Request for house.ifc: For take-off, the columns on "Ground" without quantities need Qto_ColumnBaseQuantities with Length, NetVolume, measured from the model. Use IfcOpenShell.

First a look at what the model holds.

```python
import ifcopenshell
import ifcopenshell.util.element
import ifcopenshell.util.unit

model = ifcopenshell.open("house.ifc")
print(model.schema)
for unit_type in ("LENGTHUNIT", "AREAUNIT", "VOLUMEUNIT"):
    print(unit_type, ifcopenshell.util.unit.calculate_unit_scale(model, unit_type))
storey = next(s for s in model.by_type("IfcBuildingStorey") if s.Name == "Ground")
columns = [e for e in ifcopenshell.util.element.get_decomposition(storey) if e.is_a("IfcColumn")]
for e in sorted(columns, key=lambda e: e.id()):
    print(e.id(), e.is_a(), e.Name, list(ifcopenshell.util.element.get_psets(e, qtos_only=True)), sep=" | ")
```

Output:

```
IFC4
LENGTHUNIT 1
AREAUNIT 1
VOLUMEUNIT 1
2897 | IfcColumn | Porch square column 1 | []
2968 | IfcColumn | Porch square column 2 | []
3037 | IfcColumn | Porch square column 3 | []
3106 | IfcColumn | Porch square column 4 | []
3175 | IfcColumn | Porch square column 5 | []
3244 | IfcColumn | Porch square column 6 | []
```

```python
import ifcopenshell
import ifcopenshell.api.pset
import ifcopenshell.geom
import ifcopenshell.util.element
import ifcopenshell.util.shape
import ifcopenshell.util.unit

model = ifcopenshell.open("house.ifc")
unit_scale = ifcopenshell.util.unit.calculate_unit_scale(model)
volume_scale = ifcopenshell.util.unit.calculate_unit_scale(model, "VOLUMEUNIT")
settings = ifcopenshell.geom.settings()

storey = next(s for s in model.by_type("IfcBuildingStorey") if s.Name == "Ground")
columns = [e for e in ifcopenshell.util.element.get_decomposition(storey) if e.is_a("IfcColumn")]

for e in sorted(columns, key=lambda e: e.id()):
    if ifcopenshell.util.element.get_psets(e, qtos_only=True, should_inherit=False):
        continue
    # Geometry comes back in metres, in the element's own axes.
    shape = ifcopenshell.geom.create_shape(settings, e)
    values = {
        "Length": ifcopenshell.util.shape.get_z(shape.geometry) / unit_scale,
        "NetVolume": ifcopenshell.util.shape.get_volume(shape.geometry) / volume_scale,
    }
    qto = ifcopenshell.api.pset.add_qto(model, product=e, name="Qto_ColumnBaseQuantities")
    ifcopenshell.api.pset.edit_qto(model, qto=qto, properties=values)
    print(e.id(), {k: round(v, 3) for k, v in values.items()})

model.write("house_updated.ifc")
```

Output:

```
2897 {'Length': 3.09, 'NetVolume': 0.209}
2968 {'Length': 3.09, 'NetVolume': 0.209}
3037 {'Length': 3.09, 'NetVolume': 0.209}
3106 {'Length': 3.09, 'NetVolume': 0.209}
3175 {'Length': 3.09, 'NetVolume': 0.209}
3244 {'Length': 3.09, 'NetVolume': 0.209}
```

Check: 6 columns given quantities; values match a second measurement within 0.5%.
